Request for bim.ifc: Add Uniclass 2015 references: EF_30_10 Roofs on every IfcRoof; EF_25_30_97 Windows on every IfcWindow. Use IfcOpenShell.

First a look at what the model holds.

```python
import ifcopenshell

model = ifcopenshell.open("bim.ifc")
print(model.schema)
print("classifications:", [c.Name for c in model.by_type("IfcClassification")])
for ifc_class in ("IfcDoor", "IfcRoof", "IfcStair", "IfcWall", "IfcWindow"):
    print(ifc_class, len(model.by_type(ifc_class)))
```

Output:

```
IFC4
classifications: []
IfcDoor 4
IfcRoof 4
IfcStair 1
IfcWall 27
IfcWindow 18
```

```python
import ifcopenshell
import ifcopenshell.api.classification

model = ifcopenshell.open("bim.ifc")

system = ifcopenshell.api.classification.add_classification(model, classification="Uniclass 2015")

codes = {
    "IfcRoof": ("EF_30_10", "Roofs"),
    "IfcWindow": ("EF_25_30_97", "Windows"),
}
for ifc_class, (code, name) in codes.items():
    products = model.by_type(ifc_class)
    ifcopenshell.api.classification.add_reference(
        model, products=products, classification=system, identification=code, name=name
    )
    print(code, len(products))

model.write("bim_rev.ifc")
```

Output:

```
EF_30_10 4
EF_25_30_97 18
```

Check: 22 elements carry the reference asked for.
